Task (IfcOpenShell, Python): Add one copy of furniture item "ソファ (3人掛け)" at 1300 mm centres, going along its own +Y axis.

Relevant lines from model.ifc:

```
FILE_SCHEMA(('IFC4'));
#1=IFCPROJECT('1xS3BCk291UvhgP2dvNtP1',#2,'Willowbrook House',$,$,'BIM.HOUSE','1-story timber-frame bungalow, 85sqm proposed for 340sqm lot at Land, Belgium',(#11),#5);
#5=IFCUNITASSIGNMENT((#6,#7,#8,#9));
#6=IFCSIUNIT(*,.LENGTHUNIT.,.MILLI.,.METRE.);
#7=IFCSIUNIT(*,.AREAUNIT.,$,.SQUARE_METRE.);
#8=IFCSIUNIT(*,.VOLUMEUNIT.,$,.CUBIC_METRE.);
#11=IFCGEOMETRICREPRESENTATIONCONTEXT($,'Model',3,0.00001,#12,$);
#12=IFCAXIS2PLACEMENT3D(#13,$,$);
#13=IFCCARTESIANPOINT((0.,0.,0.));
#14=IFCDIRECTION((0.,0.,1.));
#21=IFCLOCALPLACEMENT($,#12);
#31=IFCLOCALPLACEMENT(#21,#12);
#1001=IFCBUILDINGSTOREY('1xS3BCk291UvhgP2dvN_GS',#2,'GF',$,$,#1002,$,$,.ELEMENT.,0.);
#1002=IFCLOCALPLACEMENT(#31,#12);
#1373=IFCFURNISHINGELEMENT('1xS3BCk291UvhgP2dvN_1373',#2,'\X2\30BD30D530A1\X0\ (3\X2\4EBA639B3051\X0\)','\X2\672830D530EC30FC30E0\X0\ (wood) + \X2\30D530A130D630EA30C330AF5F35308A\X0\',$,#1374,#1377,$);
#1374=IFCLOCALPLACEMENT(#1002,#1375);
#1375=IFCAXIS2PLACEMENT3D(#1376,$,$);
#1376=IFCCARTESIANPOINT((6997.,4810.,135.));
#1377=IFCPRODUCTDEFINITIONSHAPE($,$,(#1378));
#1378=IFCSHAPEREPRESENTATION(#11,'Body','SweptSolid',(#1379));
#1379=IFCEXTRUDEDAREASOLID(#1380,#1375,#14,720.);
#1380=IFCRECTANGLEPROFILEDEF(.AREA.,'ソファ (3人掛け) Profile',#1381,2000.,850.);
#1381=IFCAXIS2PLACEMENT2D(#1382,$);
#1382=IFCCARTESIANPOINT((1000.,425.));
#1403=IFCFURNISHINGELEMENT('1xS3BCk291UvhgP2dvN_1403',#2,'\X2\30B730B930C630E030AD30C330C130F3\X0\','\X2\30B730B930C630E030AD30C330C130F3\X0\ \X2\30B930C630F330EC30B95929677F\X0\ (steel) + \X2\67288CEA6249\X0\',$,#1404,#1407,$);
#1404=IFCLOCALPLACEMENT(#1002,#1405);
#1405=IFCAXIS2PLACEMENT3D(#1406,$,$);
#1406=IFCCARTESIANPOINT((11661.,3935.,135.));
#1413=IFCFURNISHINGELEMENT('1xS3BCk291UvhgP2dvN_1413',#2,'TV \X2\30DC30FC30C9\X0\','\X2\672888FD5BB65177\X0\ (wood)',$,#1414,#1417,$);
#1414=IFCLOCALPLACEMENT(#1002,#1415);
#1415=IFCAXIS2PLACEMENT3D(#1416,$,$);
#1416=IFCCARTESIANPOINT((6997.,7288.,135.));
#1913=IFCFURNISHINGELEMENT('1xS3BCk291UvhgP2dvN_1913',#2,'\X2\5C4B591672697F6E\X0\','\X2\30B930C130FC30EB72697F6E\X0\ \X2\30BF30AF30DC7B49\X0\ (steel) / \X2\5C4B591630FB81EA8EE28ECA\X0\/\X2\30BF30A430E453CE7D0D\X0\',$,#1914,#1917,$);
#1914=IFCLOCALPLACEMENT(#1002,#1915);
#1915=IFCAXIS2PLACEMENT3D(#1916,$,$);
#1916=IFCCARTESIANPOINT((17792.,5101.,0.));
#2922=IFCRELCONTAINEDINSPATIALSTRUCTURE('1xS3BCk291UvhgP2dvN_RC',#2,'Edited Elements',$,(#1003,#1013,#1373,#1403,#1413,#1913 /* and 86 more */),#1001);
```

```python
import ifcopenshell
import ifcopenshell.api.geometry
import ifcopenshell.api.root
import ifcopenshell.util.element
import ifcopenshell.util.placement
import ifcopenshell.util.unit

model = ifcopenshell.open("model.ifc")
unit_scale = ifcopenshell.util.unit.calculate_unit_scale(model)


def reuse_history(source, copy):
    """copy_class also copies each property set's owner history, people and application; keep the originals."""
    for rel in copy.IsDefinedBy:
        if rel.is_a("IfcRelDefinesByProperties") and (history := rel.RelatingPropertyDefinition.OwnerHistory):
            rel.RelatingPropertyDefinition.OwnerHistory = source.OwnerHistory
            ifcopenshell.util.element.remove_deep2(model, history)


source = model.by_guid("1xS3BCk291UvhgP2dvN_1373")
base = ifcopenshell.util.placement.get_local_placement(source.ObjectPlacement)
step = base[:3, 1] * 1.3 / unit_scale

for i in range(1, 2):
    copy = ifcopenshell.api.root.copy_class(model, product=source)
    copy.Representation = ifcopenshell.util.element.copy_deep(
        model, source.Representation, exclude=["IfcGeometricRepresentationContext", "IfcRepresentationMap"]
    )
    reuse_history(source, copy)
    matrix = base.copy()
    matrix[:3, 3] += i * step
    print("added at", matrix[:3, 3].round(3) + 0.0)
    ifcopenshell.api.geometry.edit_object_placement(model, product=copy, matrix=matrix, is_si=False)

model.write("model_v2.ifc")
```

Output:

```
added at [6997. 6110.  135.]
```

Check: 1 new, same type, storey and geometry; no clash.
